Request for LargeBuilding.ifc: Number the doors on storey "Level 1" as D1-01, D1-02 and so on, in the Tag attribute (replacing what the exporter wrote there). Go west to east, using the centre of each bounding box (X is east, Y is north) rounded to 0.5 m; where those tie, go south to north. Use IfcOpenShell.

First a look at what the model holds.

```python
import ifcopenshell
import ifcopenshell.util.element
import ifcopenshell.util.placement

model = ifcopenshell.open("LargeBuilding.ifc")
print(model.schema)
storey = next(s for s in model.by_type("IfcBuildingStorey") if s.Name == "Level 1")
doors = [e for e in ifcopenshell.util.element.get_decomposition(storey) if e.is_a("IfcDoor")]
for e in sorted(doors, key=lambda e: e.id()):
    origin = ifcopenshell.util.placement.get_local_placement(e.ObjectPlacement)[:3, 3]
    print(e.id(), e.Tag, e.Name, origin.round(2) + 0.0, sep=" | ")
```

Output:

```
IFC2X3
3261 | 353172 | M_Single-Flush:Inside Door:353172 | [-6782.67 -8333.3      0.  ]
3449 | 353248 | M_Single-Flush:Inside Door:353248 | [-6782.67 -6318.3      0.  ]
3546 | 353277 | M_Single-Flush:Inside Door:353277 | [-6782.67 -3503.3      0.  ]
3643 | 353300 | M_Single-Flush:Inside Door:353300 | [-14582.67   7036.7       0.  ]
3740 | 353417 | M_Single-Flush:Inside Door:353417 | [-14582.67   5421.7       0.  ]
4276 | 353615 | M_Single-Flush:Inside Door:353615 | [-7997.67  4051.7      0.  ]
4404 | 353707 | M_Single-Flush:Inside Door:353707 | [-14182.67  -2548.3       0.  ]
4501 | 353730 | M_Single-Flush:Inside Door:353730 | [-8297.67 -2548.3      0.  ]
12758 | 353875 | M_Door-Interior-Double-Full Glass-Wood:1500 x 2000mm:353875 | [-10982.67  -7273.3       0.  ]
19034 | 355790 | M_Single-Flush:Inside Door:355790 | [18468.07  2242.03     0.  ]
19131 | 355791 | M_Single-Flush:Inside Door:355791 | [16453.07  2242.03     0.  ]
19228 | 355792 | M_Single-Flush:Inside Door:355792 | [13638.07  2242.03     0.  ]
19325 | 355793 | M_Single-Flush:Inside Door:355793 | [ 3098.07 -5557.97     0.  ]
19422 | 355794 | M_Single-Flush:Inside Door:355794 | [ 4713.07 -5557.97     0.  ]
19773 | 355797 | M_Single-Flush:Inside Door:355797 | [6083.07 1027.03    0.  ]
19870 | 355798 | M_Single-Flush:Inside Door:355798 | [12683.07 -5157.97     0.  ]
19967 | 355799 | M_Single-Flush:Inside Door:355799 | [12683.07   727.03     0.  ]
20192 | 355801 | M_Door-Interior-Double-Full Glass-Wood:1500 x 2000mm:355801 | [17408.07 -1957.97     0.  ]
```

```python
import ifcopenshell
import ifcopenshell.geom
import ifcopenshell.util.element
import ifcopenshell.util.shape

model = ifcopenshell.open("LargeBuilding.ifc")
settings = ifcopenshell.geom.settings()
settings.set("use-world-coords", True)


def centre(element):
    shape = ifcopenshell.geom.create_shape(settings, element)
    return ifcopenshell.util.shape.get_bbox_centroid(shape.geometry)


storey = next(s for s in model.by_type("IfcBuildingStorey") if s.Name == "Level 1")
doors = [e for e in ifcopenshell.util.element.get_decomposition(storey) if e.is_a("IfcDoor")]

# Insertion points can sit at a corner or the storey origin, so sort by the geometry (in metres).
centres = {e: centre(e) for e in doors}
doors.sort(key=lambda e: (round(centres[e][0] / 0.5), centres[e][1]))

for i, e in enumerate(doors, start=1):
    number = f"D1-{i:02d}"
    e.Tag = number
    print(e.id(), number)

model.write("LargeBuilding_v2.ifc")
```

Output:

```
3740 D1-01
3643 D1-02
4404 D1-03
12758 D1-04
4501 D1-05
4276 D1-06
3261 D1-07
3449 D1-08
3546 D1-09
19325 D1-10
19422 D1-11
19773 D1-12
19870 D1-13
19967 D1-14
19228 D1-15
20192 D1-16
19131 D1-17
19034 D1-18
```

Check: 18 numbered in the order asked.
